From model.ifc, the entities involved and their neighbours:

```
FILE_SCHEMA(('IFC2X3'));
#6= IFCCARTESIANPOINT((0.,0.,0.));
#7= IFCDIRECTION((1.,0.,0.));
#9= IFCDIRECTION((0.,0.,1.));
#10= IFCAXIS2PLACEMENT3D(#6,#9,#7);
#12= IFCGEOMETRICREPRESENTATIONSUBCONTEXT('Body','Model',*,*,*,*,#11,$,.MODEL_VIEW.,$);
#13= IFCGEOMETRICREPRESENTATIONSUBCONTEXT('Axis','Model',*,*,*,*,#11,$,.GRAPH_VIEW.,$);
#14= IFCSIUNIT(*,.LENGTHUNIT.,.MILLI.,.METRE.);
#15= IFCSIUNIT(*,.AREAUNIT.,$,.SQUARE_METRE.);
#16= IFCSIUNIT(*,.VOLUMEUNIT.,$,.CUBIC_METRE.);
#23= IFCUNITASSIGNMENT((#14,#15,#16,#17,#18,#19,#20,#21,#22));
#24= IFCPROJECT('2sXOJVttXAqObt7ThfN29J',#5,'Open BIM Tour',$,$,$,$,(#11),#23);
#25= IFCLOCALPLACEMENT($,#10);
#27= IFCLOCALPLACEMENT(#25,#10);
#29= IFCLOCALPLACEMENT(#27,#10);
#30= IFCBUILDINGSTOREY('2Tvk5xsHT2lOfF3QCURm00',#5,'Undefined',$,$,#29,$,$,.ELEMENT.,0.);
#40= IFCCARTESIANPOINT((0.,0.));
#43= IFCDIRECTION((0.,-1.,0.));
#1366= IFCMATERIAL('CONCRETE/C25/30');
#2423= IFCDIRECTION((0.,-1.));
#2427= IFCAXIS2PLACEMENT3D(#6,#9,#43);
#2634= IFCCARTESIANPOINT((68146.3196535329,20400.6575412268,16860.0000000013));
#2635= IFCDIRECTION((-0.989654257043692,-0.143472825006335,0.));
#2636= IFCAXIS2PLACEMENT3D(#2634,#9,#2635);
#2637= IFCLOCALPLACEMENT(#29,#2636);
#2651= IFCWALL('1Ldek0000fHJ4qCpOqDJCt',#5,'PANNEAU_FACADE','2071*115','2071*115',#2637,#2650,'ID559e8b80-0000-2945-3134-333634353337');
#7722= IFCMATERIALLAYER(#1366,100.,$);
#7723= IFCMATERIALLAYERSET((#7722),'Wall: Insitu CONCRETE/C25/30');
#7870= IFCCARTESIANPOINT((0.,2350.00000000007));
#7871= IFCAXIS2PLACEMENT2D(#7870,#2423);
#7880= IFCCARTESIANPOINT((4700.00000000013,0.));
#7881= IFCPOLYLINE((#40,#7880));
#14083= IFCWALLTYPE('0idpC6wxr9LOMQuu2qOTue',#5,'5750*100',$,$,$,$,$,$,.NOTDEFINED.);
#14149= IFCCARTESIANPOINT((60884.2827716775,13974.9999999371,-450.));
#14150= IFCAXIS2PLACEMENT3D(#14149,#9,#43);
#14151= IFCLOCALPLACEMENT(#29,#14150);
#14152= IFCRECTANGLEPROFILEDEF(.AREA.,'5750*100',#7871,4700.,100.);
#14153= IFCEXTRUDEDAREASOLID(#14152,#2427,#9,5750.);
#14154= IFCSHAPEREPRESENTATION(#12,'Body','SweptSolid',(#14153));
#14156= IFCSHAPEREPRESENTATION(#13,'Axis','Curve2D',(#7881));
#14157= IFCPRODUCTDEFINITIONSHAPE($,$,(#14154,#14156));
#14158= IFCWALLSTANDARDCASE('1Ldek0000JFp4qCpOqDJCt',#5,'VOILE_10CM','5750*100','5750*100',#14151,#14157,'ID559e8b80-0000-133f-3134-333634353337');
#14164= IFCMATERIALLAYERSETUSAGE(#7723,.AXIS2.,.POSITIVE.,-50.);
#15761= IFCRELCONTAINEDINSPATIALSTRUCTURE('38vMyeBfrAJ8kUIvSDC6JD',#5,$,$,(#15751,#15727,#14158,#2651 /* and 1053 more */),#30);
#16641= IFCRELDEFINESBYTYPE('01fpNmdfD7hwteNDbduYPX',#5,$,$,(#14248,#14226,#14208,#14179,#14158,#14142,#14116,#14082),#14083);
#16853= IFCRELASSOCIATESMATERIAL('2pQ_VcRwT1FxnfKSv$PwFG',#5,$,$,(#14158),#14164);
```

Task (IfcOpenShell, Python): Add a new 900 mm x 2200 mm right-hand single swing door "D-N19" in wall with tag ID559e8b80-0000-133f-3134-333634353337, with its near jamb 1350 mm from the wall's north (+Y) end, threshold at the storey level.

```python
import numpy as np
import ifcopenshell
import ifcopenshell.api.feature
import ifcopenshell.api.geometry
import ifcopenshell.api.root
import ifcopenshell.api.spatial
import ifcopenshell.api.type
import ifcopenshell.geom
import ifcopenshell.util.element
import ifcopenshell.util.placement
import ifcopenshell.util.representation
import ifcopenshell.util.shape
import ifcopenshell.util.unit

model = ifcopenshell.open("model.ifc")
unit_scale = ifcopenshell.util.unit.calculate_unit_scale(model)
settings = ifcopenshell.geom.settings()


def volume(element):
    """Net volume in cubic metres, openings subtracted."""
    shape = ifcopenshell.geom.create_shape(settings, element)
    return ifcopenshell.util.shape.get_volume(shape.geometry)


wall = model.by_guid("1Ldek0000JFp4qCpOqDJCt")
storey = ifcopenshell.util.element.get_container(wall, ifc_class="IfcBuildingStorey")
context = ifcopenshell.util.representation.get_context(model, "Model", "Body", "MODEL_VIEW")
before = volume(wall)

width, height, from_end, sill = 0.9, 2.2, 1.35, 0.0  # metres

# The wall runs along its own X axis, and the end named is its -X end.
wall_shape = ifcopenshell.geom.create_shape(settings, wall)
x, y, z = ifcopenshell.util.shape.get_vertices(wall_shape.geometry).T
start = x.min() + from_end
face, thickness = float(y.min()), float(y.max() - y.min())
wall_matrix = ifcopenshell.util.placement.get_local_placement(wall.ObjectPlacement)
level = ifcopenshell.util.placement.get_local_placement(storey.ObjectPlacement)[2, 3]


def in_wall(x, y):
    """Placement at x, y metres in the wall's axes, at sill height."""
    matrix = wall_matrix.copy()
    matrix[:, 3] = wall_matrix @ np.array([x / unit_scale, y / unit_scale, 0.0, 1.0])
    matrix[2, 3] = level + sill / unit_scale
    return matrix


# Opening: a box that overshoots both wall faces by 50 mm.
opening = ifcopenshell.api.root.create_entity(model, ifc_class="IfcOpeningElement")
box = ifcopenshell.api.geometry.add_wall_representation(
    model, context=context, length=width, height=height, thickness=thickness + 0.1
)
ifcopenshell.api.geometry.assign_representation(model, product=opening, representation=box)
ifcopenshell.api.geometry.edit_object_placement(model, product=opening, matrix=in_wall(start, face - 0.05), is_si=False)
ifcopenshell.api.feature.add_feature(model, feature=opening, element=wall)

door = ifcopenshell.api.root.create_entity(model, ifc_class="IfcDoor", name="D-N19")
door.OverallWidth, door.OverallHeight = width / unit_scale, height / unit_scale
body = ifcopenshell.api.geometry.add_door_representation(
    model,
    context=context,
    overall_width=door.OverallWidth,
    overall_height=door.OverallHeight,
    operation_type="SINGLE_SWING_RIGHT",
    lining_properties={"LiningDepth": thickness / unit_scale, "ThresholdDepth": thickness / unit_scale},
)
ifcopenshell.api.geometry.assign_representation(model, product=door, representation=body)
ifcopenshell.api.spatial.assign_container(model, products=[door], relating_structure=storey)
fills = ifcopenshell.api.feature.add_filling(model, opening=opening, element=door)
fills.OwnerHistory = door.OwnerHistory  # required in IFC2X3

# IFC2X3 keeps the operation on the door style.
style = ifcopenshell.api.root.create_entity(model, ifc_class="IfcDoorStyle", name="D-N19")
style.OperationType, style.ConstructionType = "SINGLE_SWING_RIGHT", "NOTDEFINED"
style.ParameterTakesPrecedence = style.Sizeable = False
ifcopenshell.api.type.assign_type(model, related_objects=[door], relating_type=style)

# The lining spans the wall, so the door starts at the wall face.
ifcopenshell.api.geometry.edit_object_placement(model, product=door, matrix=in_wall(start, face), is_si=False)

after = volume(wall)

print(f"wall volume {before:.3f} -> {after:.3f} m3")

model.write("model_rev.ifc")
```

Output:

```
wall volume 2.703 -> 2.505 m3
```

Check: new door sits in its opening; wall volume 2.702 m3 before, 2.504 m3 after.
